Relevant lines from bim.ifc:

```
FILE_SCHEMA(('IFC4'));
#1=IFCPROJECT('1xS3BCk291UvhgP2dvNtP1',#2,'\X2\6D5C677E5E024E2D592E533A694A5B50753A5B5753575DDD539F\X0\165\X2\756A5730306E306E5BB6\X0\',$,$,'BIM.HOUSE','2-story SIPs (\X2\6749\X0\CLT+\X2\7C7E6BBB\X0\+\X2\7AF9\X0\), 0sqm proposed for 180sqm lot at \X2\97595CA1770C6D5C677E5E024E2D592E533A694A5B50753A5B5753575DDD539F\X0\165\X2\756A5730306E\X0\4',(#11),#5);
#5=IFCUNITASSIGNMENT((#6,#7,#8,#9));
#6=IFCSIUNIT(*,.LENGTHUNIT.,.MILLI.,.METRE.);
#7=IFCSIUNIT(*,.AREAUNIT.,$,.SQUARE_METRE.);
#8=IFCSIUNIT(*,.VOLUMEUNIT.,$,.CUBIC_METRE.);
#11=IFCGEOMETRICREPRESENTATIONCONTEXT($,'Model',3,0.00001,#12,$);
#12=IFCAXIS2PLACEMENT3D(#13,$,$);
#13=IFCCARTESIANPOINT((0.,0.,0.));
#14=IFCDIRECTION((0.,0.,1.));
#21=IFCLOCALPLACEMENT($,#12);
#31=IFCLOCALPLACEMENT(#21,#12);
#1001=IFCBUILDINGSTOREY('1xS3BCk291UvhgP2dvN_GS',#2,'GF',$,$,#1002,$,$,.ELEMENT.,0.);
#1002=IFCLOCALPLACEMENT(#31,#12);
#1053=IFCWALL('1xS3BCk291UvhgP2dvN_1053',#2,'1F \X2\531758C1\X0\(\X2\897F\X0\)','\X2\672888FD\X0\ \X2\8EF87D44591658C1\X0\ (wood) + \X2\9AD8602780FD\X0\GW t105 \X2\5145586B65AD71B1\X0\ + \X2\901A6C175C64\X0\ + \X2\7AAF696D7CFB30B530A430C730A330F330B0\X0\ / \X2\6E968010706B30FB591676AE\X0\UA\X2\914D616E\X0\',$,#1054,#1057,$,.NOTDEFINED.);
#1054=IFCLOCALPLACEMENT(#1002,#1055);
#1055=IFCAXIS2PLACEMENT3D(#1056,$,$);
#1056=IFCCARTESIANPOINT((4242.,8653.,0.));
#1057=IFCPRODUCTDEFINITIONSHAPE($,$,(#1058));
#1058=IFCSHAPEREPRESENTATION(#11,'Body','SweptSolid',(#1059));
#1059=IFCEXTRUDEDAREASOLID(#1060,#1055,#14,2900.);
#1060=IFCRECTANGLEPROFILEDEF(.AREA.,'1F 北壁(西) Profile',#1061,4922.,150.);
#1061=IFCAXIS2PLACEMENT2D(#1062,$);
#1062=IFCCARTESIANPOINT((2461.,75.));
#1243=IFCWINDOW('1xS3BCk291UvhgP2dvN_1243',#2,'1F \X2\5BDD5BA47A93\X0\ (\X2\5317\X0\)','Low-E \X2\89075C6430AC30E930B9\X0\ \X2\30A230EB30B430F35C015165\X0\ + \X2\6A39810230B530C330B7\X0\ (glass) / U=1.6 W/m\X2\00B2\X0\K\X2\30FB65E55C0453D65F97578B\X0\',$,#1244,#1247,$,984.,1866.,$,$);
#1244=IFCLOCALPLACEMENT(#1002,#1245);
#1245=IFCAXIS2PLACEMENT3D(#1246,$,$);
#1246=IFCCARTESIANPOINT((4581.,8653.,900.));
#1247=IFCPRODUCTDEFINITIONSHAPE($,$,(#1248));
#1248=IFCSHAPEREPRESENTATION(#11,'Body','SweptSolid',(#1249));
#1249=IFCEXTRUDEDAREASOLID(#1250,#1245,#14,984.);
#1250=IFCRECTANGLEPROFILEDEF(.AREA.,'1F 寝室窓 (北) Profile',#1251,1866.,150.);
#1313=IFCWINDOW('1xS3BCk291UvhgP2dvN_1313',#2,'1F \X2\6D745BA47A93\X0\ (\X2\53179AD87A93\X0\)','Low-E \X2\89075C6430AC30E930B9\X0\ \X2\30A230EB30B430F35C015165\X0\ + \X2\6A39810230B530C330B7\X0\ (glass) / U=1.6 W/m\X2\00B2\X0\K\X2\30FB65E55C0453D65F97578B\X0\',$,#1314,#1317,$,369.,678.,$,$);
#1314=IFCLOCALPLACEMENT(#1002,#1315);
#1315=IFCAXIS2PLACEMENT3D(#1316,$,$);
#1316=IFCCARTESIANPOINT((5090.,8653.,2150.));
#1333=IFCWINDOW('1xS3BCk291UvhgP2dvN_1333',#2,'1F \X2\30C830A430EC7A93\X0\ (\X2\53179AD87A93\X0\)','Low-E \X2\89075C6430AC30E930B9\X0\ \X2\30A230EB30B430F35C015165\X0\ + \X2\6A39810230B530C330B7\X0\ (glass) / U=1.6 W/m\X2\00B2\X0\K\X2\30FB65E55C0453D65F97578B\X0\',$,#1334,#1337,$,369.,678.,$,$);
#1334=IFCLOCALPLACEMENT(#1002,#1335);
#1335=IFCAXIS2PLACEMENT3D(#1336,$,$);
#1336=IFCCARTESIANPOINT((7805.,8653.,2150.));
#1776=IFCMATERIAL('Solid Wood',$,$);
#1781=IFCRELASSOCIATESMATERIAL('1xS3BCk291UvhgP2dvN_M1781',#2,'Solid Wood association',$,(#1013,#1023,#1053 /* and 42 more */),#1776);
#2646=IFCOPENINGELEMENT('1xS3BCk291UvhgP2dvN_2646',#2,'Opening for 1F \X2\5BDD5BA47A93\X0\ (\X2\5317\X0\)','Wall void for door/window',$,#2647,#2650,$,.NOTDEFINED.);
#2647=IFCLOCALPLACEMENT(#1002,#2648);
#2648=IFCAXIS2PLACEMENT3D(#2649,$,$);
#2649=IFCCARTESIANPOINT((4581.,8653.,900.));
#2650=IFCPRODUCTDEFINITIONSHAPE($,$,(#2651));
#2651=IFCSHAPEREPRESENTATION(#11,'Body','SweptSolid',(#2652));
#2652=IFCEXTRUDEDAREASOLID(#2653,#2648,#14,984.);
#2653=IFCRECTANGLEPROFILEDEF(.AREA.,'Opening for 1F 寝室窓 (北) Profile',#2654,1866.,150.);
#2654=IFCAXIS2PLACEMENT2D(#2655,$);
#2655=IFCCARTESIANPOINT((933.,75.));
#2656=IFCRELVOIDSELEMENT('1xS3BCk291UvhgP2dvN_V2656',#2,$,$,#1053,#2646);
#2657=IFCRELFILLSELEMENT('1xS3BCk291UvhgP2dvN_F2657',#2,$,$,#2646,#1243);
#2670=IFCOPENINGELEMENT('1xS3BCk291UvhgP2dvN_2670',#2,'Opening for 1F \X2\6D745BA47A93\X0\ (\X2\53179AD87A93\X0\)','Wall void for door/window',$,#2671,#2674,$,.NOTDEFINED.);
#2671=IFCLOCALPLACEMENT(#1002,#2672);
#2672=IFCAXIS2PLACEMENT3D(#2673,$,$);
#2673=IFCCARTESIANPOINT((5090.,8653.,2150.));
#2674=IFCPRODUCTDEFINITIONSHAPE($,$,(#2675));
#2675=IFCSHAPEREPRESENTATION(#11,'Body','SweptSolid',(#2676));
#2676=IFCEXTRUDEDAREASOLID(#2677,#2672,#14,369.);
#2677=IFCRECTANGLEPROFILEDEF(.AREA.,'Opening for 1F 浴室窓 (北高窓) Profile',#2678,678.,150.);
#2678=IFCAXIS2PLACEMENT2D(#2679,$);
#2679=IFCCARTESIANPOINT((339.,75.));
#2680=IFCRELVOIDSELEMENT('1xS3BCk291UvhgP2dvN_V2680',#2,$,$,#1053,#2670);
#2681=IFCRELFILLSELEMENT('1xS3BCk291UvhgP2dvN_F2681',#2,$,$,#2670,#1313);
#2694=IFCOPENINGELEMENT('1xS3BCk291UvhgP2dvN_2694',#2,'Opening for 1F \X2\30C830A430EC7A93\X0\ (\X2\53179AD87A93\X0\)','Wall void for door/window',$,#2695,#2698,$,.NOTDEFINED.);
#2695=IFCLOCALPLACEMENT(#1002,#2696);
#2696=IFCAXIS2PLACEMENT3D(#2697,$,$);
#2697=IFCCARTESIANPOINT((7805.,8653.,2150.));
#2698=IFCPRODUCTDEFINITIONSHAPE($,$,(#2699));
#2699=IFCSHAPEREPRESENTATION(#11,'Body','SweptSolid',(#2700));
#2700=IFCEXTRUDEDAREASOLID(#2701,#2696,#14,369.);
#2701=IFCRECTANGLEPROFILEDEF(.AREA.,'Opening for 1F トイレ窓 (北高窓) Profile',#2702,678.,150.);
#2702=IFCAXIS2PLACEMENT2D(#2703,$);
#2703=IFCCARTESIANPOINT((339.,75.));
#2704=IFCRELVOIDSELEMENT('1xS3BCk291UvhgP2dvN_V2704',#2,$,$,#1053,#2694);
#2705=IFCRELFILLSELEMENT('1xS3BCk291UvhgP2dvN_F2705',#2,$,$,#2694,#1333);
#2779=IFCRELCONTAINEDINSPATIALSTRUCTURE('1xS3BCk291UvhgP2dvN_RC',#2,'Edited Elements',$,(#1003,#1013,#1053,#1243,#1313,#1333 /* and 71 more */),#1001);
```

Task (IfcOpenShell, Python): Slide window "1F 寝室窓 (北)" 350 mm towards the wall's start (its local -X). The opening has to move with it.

```python
import ifcopenshell
import ifcopenshell.api.geometry
import ifcopenshell.util.placement

model = ifcopenshell.open("bim.ifc")

window = model.by_id(1243)
opening = window.FillsVoids[0].RelatingOpeningElement
wall = opening.VoidsElements[0].RelatingBuildingElement

wall_matrix = ifcopenshell.util.placement.get_local_placement(wall.ObjectPlacement)
shift = wall_matrix[:3, 0] * -350.0
before = ifcopenshell.util.placement.get_local_placement(window.ObjectPlacement)[:3, 3].copy()

# The window is not placed relative to its opening, so move both.
for product in (opening, window):
    matrix = ifcopenshell.util.placement.get_local_placement(product.ObjectPlacement)
    matrix[:3, 3] += shift
    ifcopenshell.api.geometry.edit_object_placement(model, product=product, matrix=matrix, is_si=False)

after = ifcopenshell.util.placement.get_local_placement(window.ObjectPlacement)[:3, 3]
print("window moved by", (after - before).round(3) + 0.0)

model.write("bim_edited.ifc")
```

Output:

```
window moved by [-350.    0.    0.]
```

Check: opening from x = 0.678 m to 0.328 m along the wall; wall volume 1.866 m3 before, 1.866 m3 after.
